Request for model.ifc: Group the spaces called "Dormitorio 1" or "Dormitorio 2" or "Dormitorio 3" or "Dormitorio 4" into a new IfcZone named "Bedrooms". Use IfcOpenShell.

First a look at what the model holds.

```python
import ifcopenshell

model = ifcopenshell.open("model.ifc")
print(model.schema)
seen = {}
for space in model.by_type("IfcSpace"):
    seen[space.LongName] = seen.get(space.LongName, 0) + 1
for name, count in sorted(seen.items(), key=str):
    print(count, "x", name)
print("zones:", [z.Name for z in model.by_type("IfcZone")][:20])
```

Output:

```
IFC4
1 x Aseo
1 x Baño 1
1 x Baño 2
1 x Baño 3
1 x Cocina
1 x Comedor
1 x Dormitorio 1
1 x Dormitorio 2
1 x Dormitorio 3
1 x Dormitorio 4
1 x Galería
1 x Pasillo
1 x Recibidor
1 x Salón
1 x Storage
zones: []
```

```python
import ifcopenshell
import ifcopenshell.api.group
import ifcopenshell.api.root

model = ifcopenshell.open("model.ifc")

names = {"Dormitorio 1", "Dormitorio 2", "Dormitorio 3", "Dormitorio 4"}
spaces = [s for s in model.by_type("IfcSpace") if s.LongName in names]

zone = ifcopenshell.api.root.create_entity(model, ifc_class="IfcZone", name="Bedrooms")
ifcopenshell.api.group.assign_group(model, products=spaces, group=zone)
print(len(spaces), "spaces in", zone.Name)

model.write("model_edited.ifc")
```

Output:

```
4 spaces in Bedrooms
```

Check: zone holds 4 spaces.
